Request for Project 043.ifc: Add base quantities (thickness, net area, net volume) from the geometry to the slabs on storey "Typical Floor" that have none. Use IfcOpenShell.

First a look at what the model holds.

```python
import ifcopenshell
import ifcopenshell.util.element
import ifcopenshell.util.unit

model = ifcopenshell.open("Project 043.ifc")
print(model.schema)
for unit_type in ("LENGTHUNIT", "AREAUNIT", "VOLUMEUNIT"):
    print(unit_type, ifcopenshell.util.unit.calculate_unit_scale(model, unit_type))
storey = next(s for s in model.by_type("IfcBuildingStorey") if s.Name == "Typical Floor")
slabs = [e for e in ifcopenshell.util.element.get_decomposition(storey) if e.is_a("IfcSlab")]
for e in sorted(slabs, key=lambda e: e.id()):
    print(e.id(), e.is_a(), e.Name, list(ifcopenshell.util.element.get_psets(e, qtos_only=True)), sep=" | ")
```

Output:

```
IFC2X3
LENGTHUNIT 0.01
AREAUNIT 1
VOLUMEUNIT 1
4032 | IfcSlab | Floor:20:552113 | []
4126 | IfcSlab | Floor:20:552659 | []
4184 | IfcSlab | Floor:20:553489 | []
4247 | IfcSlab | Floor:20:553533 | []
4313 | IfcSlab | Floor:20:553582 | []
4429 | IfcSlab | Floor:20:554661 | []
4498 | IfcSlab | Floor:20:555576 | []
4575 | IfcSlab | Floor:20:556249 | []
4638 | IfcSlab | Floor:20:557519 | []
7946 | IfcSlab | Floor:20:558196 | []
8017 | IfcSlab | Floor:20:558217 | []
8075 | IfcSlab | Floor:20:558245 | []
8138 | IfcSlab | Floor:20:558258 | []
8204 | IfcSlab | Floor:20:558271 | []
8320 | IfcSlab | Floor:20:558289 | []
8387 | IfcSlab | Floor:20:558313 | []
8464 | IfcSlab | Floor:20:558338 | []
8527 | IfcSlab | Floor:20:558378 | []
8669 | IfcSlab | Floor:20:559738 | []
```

```python
import ifcopenshell
import ifcopenshell.api.pset
import ifcopenshell.geom
import ifcopenshell.util.element
import ifcopenshell.util.shape
import ifcopenshell.util.unit

model = ifcopenshell.open("Project 043.ifc")
unit_scale = ifcopenshell.util.unit.calculate_unit_scale(model)
area_scale = ifcopenshell.util.unit.calculate_unit_scale(model, "AREAUNIT")
volume_scale = ifcopenshell.util.unit.calculate_unit_scale(model, "VOLUMEUNIT")
settings = ifcopenshell.geom.settings()

storey = next(s for s in model.by_type("IfcBuildingStorey") if s.Name == "Typical Floor")
slabs = [e for e in ifcopenshell.util.element.get_decomposition(storey) if e.is_a("IfcSlab")]

for e in sorted(slabs, key=lambda e: e.id()):
    if ifcopenshell.util.element.get_psets(e, qtos_only=True, should_inherit=False):
        continue
    # Geometry comes back in metres, in the element's own axes.
    shape = ifcopenshell.geom.create_shape(settings, e)
    values = {
        "Width": ifcopenshell.util.shape.get_z(shape.geometry) / unit_scale,
        "NetArea": ifcopenshell.util.shape.get_footprint_area(shape.geometry) / area_scale,
        "NetVolume": ifcopenshell.util.shape.get_volume(shape.geometry) / volume_scale,
    }
    qto = ifcopenshell.api.pset.add_qto(model, product=e, name="BaseQuantities")
    ifcopenshell.api.pset.edit_qto(model, qto=qto, properties=values)
    print(e.id(), {k: round(v, 3) for k, v in values.items()})

model.write("Project 043_v2.ifc")
```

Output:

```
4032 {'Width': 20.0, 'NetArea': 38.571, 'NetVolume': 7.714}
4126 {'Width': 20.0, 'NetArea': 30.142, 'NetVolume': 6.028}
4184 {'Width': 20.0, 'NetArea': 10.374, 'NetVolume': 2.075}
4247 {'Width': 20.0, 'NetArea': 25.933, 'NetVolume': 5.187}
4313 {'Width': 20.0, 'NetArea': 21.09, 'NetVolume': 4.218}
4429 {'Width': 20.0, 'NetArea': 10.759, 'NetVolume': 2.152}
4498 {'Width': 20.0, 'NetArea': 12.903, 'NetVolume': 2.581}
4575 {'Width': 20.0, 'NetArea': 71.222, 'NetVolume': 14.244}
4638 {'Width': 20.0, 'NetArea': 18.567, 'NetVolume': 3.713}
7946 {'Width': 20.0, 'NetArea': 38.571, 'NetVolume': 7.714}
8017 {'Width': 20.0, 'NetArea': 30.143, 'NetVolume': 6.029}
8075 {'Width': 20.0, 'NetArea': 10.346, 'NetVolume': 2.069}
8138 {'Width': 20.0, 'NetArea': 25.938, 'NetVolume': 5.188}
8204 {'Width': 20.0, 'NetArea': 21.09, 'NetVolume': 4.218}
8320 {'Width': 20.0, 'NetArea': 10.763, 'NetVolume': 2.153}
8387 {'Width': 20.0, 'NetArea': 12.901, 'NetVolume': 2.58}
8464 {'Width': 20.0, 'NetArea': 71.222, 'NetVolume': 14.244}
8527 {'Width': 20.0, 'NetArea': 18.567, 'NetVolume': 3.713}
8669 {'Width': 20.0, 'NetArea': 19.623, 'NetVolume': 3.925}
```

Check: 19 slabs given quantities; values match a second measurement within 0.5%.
